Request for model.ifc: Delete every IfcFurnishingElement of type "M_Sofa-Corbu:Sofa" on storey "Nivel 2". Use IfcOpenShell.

First a look at what the model holds.

```python
import ifcopenshell
import ifcopenshell.util.element

model = ifcopenshell.open("model.ifc")
print(model.schema)
storey = next(s for s in model.by_type("IfcBuildingStorey") if s.Name == "Nivel 2")
furniture = [e for e in ifcopenshell.util.element.get_decomposition(storey) if e.is_a("IfcFurnishingElement")]
seen = {}
for e in furniture:
    element_type = ifcopenshell.util.element.get_type(e)
    name = element_type.Name if element_type not in (None, e) else None
    seen[name] = seen.get(name, 0) + 1
for name, count in sorted(seen.items(), key=str):
    print(count, "x", name)
```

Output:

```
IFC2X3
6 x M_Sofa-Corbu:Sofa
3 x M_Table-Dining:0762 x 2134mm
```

```python
import ifcopenshell
import ifcopenshell.api.root
import ifcopenshell.util.element

model = ifcopenshell.open("model.ifc")

storey = next(s for s in model.by_type("IfcBuildingStorey") if s.Name == "Nivel 2")
furniture = [e for e in ifcopenshell.util.element.get_decomposition(storey) if e.is_a("IfcFurnishingElement")]
targets = [e for e in furniture if (t := ifcopenshell.util.element.get_type(e)) not in (None, e) and t.Name == "M_Sofa-Corbu:Sofa"]

for e in targets:
    ifcopenshell.api.root.remove_product(model, product=e)
print(len(targets), "removed")

model.write("model_rev.ifc")
```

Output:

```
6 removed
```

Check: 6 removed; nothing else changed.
